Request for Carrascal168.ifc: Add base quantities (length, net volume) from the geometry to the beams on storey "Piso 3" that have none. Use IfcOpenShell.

First a look at what the model holds.

```python
import ifcopenshell
import ifcopenshell.util.element
import ifcopenshell.util.unit

model = ifcopenshell.open("Carrascal168.ifc")
print(model.schema)
for unit_type in ("LENGTHUNIT", "AREAUNIT", "VOLUMEUNIT"):
    print(unit_type, ifcopenshell.util.unit.calculate_unit_scale(model, unit_type))
storey = next(s for s in model.by_type("IfcBuildingStorey") if s.Name == "Piso 3")
beams = [e for e in ifcopenshell.util.element.get_decomposition(storey) if e.is_a("IfcBeam")]
for e in sorted(beams, key=lambda e: e.id()):
    print(e.id(), e.is_a(), e.Name, list(ifcopenshell.util.element.get_psets(e, qtos_only=True)), sep=" | ")
```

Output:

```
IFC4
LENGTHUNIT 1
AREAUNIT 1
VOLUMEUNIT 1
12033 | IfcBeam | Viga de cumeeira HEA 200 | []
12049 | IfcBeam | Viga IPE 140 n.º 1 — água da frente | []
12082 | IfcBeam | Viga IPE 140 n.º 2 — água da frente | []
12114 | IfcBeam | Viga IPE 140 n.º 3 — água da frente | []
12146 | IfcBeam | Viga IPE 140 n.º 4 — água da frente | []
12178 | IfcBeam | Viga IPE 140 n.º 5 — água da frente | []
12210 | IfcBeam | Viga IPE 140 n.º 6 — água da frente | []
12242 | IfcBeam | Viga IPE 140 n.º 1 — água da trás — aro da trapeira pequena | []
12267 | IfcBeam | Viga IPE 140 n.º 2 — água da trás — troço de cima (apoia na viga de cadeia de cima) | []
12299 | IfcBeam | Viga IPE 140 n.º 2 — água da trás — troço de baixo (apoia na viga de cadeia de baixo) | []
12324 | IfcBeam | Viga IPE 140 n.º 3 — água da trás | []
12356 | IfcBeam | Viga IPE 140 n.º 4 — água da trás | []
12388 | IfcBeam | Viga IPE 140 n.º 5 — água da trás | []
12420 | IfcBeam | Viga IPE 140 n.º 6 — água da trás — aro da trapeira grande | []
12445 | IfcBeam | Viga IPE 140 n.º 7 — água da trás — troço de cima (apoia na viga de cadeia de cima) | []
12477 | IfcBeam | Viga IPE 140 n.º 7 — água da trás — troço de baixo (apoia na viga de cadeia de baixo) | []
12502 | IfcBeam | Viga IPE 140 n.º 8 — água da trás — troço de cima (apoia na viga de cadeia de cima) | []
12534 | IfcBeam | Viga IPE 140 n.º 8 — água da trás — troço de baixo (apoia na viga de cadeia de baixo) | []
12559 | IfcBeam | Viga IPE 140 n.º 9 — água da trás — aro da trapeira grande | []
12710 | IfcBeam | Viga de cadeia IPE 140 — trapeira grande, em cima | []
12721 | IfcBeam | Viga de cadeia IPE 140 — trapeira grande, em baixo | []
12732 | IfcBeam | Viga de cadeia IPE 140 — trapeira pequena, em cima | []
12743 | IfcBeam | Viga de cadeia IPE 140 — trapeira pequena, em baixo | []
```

```python
import ifcopenshell
import ifcopenshell.api.pset
import ifcopenshell.geom
import ifcopenshell.util.element
import ifcopenshell.util.shape
import ifcopenshell.util.unit

model = ifcopenshell.open("Carrascal168.ifc")
unit_scale = ifcopenshell.util.unit.calculate_unit_scale(model)
volume_scale = ifcopenshell.util.unit.calculate_unit_scale(model, "VOLUMEUNIT")
settings = ifcopenshell.geom.settings()

storey = next(s for s in model.by_type("IfcBuildingStorey") if s.Name == "Piso 3")
beams = [e for e in ifcopenshell.util.element.get_decomposition(storey) if e.is_a("IfcBeam")]

for e in sorted(beams, key=lambda e: e.id()):
    if ifcopenshell.util.element.get_psets(e, qtos_only=True, should_inherit=False):
        continue
    # Geometry comes back in metres, in the element's own axes.
    shape = ifcopenshell.geom.create_shape(settings, e)
    values = {
        "Length": ifcopenshell.util.shape.get_max_xyz(shape.geometry) / unit_scale,
        "NetVolume": ifcopenshell.util.shape.get_volume(shape.geometry) / volume_scale,
    }
    qto = ifcopenshell.api.pset.add_qto(model, product=e, name="Qto_BeamBaseQuantities")
    ifcopenshell.api.pset.edit_qto(model, qto=qto, properties=values)
    print(e.id(), {k: round(v, 3) for k, v in values.items()})

model.write("Carrascal168_updated.ifc")
```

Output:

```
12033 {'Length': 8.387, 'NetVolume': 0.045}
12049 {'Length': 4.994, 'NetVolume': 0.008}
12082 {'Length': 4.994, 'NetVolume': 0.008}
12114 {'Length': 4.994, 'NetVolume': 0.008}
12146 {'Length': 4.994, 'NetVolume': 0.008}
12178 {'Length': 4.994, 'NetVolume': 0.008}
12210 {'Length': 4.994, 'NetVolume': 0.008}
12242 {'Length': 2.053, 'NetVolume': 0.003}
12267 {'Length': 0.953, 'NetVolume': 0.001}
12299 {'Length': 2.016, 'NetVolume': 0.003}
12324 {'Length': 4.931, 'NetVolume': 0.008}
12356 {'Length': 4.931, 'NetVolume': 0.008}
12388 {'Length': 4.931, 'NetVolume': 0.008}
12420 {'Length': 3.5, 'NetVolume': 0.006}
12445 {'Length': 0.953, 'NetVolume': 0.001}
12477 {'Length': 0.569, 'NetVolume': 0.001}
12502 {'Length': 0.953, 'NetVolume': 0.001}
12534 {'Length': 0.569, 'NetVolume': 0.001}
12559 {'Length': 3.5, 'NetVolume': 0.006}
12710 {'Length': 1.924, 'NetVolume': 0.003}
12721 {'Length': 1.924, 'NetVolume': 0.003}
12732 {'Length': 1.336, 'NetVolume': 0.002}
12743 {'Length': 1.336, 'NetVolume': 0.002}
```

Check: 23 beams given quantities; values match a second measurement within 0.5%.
